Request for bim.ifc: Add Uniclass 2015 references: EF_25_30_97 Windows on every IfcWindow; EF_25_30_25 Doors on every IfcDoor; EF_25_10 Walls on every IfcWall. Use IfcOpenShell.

First a look at what the model holds.

```python
import ifcopenshell

model = ifcopenshell.open("bim.ifc")
print(model.schema)
print("classifications:", [c.Name for c in model.by_type("IfcClassification")])
for ifc_class in ("IfcDoor", "IfcRoof", "IfcStair", "IfcWall", "IfcWindow"):
    print(ifc_class, len(model.by_type(ifc_class)))
```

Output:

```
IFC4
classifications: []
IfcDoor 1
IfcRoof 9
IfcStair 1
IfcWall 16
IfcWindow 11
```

```python
import ifcopenshell
import ifcopenshell.api.classification

model = ifcopenshell.open("bim.ifc")

system = ifcopenshell.api.classification.add_classification(model, classification="Uniclass 2015")

codes = {
    "IfcWindow": ("EF_25_30_97", "Windows"),
    "IfcDoor": ("EF_25_30_25", "Doors"),
    "IfcWall": ("EF_25_10", "Walls"),
}
for ifc_class, (code, name) in codes.items():
    products = model.by_type(ifc_class)
    ifcopenshell.api.classification.add_reference(
        model, products=products, classification=system, identification=code, name=name
    )
    print(code, len(products))

model.write("bim-out.ifc")
```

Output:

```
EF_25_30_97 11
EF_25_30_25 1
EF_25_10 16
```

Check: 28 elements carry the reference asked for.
